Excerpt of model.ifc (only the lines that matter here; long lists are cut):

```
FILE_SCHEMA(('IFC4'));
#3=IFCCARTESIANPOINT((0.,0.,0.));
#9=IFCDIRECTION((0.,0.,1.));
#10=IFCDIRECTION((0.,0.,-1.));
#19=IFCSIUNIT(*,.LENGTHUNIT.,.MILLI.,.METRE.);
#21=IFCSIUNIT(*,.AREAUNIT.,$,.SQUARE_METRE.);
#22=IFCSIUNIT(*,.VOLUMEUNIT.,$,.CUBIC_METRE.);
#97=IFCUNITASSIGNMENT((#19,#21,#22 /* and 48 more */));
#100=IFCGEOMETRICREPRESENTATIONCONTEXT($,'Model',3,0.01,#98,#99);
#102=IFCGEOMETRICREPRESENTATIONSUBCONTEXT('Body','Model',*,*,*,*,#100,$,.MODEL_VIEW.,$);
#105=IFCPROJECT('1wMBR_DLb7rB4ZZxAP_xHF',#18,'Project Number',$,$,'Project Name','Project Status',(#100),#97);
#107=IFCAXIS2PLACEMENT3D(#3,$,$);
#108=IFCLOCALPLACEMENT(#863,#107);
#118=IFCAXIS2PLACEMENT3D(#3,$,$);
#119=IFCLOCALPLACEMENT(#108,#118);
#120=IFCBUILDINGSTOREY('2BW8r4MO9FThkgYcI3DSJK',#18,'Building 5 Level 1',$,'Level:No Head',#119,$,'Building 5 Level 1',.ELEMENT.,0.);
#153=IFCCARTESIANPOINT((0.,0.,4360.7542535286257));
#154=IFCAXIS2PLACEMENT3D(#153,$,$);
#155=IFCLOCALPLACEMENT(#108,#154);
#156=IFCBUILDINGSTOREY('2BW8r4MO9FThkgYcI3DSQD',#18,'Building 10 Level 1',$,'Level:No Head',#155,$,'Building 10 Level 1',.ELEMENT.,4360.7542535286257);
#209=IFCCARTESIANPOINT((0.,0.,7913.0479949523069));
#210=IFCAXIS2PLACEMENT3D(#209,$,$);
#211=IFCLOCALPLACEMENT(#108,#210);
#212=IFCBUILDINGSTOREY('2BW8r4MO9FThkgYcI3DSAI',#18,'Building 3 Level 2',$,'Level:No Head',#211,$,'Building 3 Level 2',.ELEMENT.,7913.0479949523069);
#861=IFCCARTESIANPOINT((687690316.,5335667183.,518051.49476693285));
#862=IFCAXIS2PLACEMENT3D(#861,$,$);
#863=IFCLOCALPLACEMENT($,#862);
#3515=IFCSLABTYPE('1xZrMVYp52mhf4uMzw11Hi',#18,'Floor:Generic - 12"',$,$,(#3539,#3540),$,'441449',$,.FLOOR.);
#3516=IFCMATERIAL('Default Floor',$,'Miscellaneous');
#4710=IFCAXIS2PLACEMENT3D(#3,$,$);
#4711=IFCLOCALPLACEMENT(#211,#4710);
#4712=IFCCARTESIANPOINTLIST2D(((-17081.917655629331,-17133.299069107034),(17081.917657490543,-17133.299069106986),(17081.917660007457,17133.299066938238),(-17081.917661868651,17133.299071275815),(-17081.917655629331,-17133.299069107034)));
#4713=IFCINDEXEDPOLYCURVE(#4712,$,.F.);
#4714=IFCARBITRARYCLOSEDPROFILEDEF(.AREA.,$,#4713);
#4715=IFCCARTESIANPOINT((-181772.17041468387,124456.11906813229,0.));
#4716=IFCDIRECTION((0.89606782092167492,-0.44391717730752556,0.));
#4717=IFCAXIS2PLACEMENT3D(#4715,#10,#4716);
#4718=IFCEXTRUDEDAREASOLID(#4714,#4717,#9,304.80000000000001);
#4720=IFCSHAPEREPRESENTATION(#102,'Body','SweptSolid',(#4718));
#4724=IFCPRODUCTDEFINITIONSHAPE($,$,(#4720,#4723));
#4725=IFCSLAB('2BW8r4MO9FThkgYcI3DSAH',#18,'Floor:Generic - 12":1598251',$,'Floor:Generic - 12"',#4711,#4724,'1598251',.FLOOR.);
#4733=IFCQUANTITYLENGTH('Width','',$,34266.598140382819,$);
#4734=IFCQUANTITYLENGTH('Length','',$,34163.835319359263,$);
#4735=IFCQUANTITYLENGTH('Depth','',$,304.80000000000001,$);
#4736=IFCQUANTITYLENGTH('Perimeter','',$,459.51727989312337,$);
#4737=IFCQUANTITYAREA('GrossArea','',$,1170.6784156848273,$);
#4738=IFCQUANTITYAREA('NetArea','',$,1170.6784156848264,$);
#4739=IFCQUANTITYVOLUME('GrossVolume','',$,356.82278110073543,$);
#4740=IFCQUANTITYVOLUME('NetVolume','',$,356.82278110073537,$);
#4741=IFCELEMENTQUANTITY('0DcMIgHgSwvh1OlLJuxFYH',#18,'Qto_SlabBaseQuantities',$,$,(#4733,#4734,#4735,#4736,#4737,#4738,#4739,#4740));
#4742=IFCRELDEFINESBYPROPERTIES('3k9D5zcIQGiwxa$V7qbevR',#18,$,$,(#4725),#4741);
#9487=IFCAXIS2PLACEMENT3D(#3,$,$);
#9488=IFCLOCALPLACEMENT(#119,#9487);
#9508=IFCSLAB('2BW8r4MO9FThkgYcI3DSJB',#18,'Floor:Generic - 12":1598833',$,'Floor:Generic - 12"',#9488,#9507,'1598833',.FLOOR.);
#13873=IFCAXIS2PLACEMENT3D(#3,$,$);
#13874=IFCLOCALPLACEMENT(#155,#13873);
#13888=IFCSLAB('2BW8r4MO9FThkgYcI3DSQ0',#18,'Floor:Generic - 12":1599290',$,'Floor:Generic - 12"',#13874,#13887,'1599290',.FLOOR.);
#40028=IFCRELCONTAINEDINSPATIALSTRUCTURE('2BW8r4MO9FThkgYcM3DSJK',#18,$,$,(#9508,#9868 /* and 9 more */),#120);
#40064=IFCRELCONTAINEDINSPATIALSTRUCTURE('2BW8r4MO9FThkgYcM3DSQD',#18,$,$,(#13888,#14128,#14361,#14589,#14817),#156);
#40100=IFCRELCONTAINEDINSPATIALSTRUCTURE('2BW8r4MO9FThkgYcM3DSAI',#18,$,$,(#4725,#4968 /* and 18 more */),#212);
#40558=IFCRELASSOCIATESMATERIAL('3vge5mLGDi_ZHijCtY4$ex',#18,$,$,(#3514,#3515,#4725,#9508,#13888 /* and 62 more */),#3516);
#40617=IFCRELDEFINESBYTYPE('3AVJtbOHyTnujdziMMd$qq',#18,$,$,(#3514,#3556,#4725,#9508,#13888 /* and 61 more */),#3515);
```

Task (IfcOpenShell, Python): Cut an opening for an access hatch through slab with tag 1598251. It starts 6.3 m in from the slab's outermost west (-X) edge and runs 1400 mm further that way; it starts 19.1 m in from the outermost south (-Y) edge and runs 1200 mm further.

```python
import numpy as np
import ifcopenshell
import ifcopenshell.api.feature
import ifcopenshell.api.geometry
import ifcopenshell.api.pset
import ifcopenshell.api.root
import ifcopenshell.geom
import ifcopenshell.util.element
import ifcopenshell.util.placement
import ifcopenshell.util.representation
import ifcopenshell.util.shape
import ifcopenshell.util.unit

model = ifcopenshell.open("model.ifc")
unit_scale = ifcopenshell.util.unit.calculate_unit_scale(model)
area_scale = ifcopenshell.util.unit.calculate_unit_scale(model, "AREAUNIT")
volume_scale = ifcopenshell.util.unit.calculate_unit_scale(model, "VOLUMEUNIT")
settings = ifcopenshell.geom.settings()


def volume(element):
    """Net volume in cubic metres, openings subtracted."""
    shape = ifcopenshell.geom.create_shape(settings, element)
    return ifcopenshell.util.shape.get_volume(shape.geometry)


slab = model.by_guid("2BW8r4MO9FThkgYcI3DSAH")
before = volume(slab)

# Extent in the slab's own axes, in metres. The edges named are its -X and -Y sides.
slab_shape = ifcopenshell.geom.create_shape(settings, slab)
vertices = ifcopenshell.util.shape.get_vertices(slab_shape.geometry)
x_min, y_min, bottom = vertices.min(axis=0)
top = vertices[:, 2].max()

opening = ifcopenshell.api.root.create_entity(model, ifc_class="IfcOpeningElement", name="Access hatch opening", predefined_type="OPENING")
context = ifcopenshell.util.representation.get_context(model, "Model", "Body", "MODEL_VIEW")
width, depth = 1.4, 1.2
outline = [(0.0, 0.0), (width, 0.0), (width, depth), (0.0, depth), (0.0, 0.0)]
# Overshoot both faces by 50 mm so the cut is clean.
shape = ifcopenshell.api.geometry.add_slab_representation(
    model, context=context, depth=top - bottom + 0.1, polyline=outline
)
ifcopenshell.api.geometry.assign_representation(model, product=opening, representation=shape)

matrix = ifcopenshell.util.placement.get_local_placement(slab.ObjectPlacement)
matrix[:, 3] = matrix @ np.append(np.array([x_min + 6.3, y_min + 19.1, bottom - 0.05]) / unit_scale, 1.0)
ifcopenshell.api.geometry.edit_object_placement(model, product=opening, matrix=matrix, is_si=False)
ifcopenshell.api.feature.add_feature(model, feature=opening, element=slab)

after = volume(slab)

# Update the slab's stored quantities.
qto = model.by_id(ifcopenshell.util.element.get_pset(slab, "Qto_SlabBaseQuantities", should_inherit=False)["id"])
ifcopenshell.api.pset.edit_qto(model, qto=qto, properties={
    "NetArea": after / (top - bottom) / area_scale,
    "NetVolume": after / volume_scale,
})

print(f"slab volume {before:.3f} -> {after:.3f} m3")

model.write("model_rev.ifc")
```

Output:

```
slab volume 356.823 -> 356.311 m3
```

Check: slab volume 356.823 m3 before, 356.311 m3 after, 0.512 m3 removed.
